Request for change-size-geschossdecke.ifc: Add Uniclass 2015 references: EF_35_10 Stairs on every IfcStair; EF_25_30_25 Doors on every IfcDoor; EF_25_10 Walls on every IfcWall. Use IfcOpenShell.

First a look at what the model holds.

```python
import ifcopenshell

model = ifcopenshell.open("change-size-geschossdecke.ifc")
print(model.schema)
print("classifications:", [c.Name for c in model.by_type("IfcClassification")])
for ifc_class in ("IfcDoor", "IfcRoof", "IfcStair", "IfcWall", "IfcWindow"):
    print(ifc_class, len(model.by_type(ifc_class)))
```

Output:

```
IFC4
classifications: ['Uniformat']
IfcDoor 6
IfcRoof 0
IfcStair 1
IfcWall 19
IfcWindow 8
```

```python
import ifcopenshell
import ifcopenshell.api.classification

model = ifcopenshell.open("change-size-geschossdecke.ifc")

system = ifcopenshell.api.classification.add_classification(model, classification="Uniclass 2015")

codes = {
    "IfcStair": ("EF_35_10", "Stairs"),
    "IfcDoor": ("EF_25_30_25", "Doors"),
    "IfcWall": ("EF_25_10", "Walls"),
}
for ifc_class, (code, name) in codes.items():
    products = model.by_type(ifc_class)
    ifcopenshell.api.classification.add_reference(
        model, products=products, classification=system, identification=code, name=name
    )
    print(code, len(products))

model.write("change-size-geschossdecke_updated.ifc")
```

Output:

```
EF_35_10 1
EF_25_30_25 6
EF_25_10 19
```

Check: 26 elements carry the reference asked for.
